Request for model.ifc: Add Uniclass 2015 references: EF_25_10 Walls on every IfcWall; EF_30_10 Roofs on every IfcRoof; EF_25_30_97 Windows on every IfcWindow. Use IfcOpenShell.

First a look at what the model holds.

```python
import ifcopenshell

model = ifcopenshell.open("model.ifc")
print(model.schema)
print("classifications:", [c.Name for c in model.by_type("IfcClassification")])
for ifc_class in ("IfcDoor", "IfcRoof", "IfcStair", "IfcWall", "IfcWindow"):
    print(ifc_class, len(model.by_type(ifc_class)))
```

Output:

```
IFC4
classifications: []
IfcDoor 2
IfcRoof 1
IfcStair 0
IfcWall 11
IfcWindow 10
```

```python
import ifcopenshell
import ifcopenshell.api.classification

model = ifcopenshell.open("model.ifc")

system = ifcopenshell.api.classification.add_classification(model, classification="Uniclass 2015")

codes = {
    "IfcWall": ("EF_25_10", "Walls"),
    "IfcRoof": ("EF_30_10", "Roofs"),
    "IfcWindow": ("EF_25_30_97", "Windows"),
}
for ifc_class, (code, name) in codes.items():
    products = model.by_type(ifc_class)
    ifcopenshell.api.classification.add_reference(
        model, products=products, classification=system, identification=code, name=name
    )
    print(code, len(products))

model.write("model-out.ifc")
```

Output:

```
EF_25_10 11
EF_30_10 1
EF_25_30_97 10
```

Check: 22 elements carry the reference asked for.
